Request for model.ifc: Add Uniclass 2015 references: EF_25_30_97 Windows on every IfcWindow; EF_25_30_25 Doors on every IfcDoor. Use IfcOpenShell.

First a look at what the model holds.

```python
import ifcopenshell

model = ifcopenshell.open("model.ifc")
print(model.schema)
print("classifications:", [c.Name for c in model.by_type("IfcClassification")])
for ifc_class in ("IfcDoor", "IfcRoof", "IfcStair", "IfcWall", "IfcWindow"):
    print(ifc_class, len(model.by_type(ifc_class)))
```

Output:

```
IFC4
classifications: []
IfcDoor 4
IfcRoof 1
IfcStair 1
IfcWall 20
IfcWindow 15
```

```python
import ifcopenshell
import ifcopenshell.api.classification

model = ifcopenshell.open("model.ifc")

system = ifcopenshell.api.classification.add_classification(model, classification="Uniclass 2015")

codes = {
    "IfcWindow": ("EF_25_30_97", "Windows"),
    "IfcDoor": ("EF_25_30_25", "Doors"),
}
for ifc_class, (code, name) in codes.items():
    products = model.by_type(ifc_class)
    ifcopenshell.api.classification.add_reference(
        model, products=products, classification=system, identification=code, name=name
    )
    print(code, len(products))

model.write("model_edited.ifc")
```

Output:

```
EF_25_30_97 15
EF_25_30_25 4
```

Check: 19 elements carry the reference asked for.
